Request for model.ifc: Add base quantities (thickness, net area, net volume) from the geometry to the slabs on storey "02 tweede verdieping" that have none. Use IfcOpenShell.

First a look at what the model holds.

```python
import ifcopenshell
import ifcopenshell.util.element
import ifcopenshell.util.unit

model = ifcopenshell.open("model.ifc")
print(model.schema)
for unit_type in ("LENGTHUNIT", "AREAUNIT", "VOLUMEUNIT"):
    print(unit_type, ifcopenshell.util.unit.calculate_unit_scale(model, unit_type))
storey = next(s for s in model.by_type("IfcBuildingStorey") if s.Name == "02 tweede verdieping")
slabs = [e for e in ifcopenshell.util.element.get_decomposition(storey) if e.is_a("IfcSlab")]
for e in sorted(slabs, key=lambda e: e.id()):
    print(e.id(), e.is_a(), e.Name, list(ifcopenshell.util.element.get_psets(e, qtos_only=True)), sep=" | ")
```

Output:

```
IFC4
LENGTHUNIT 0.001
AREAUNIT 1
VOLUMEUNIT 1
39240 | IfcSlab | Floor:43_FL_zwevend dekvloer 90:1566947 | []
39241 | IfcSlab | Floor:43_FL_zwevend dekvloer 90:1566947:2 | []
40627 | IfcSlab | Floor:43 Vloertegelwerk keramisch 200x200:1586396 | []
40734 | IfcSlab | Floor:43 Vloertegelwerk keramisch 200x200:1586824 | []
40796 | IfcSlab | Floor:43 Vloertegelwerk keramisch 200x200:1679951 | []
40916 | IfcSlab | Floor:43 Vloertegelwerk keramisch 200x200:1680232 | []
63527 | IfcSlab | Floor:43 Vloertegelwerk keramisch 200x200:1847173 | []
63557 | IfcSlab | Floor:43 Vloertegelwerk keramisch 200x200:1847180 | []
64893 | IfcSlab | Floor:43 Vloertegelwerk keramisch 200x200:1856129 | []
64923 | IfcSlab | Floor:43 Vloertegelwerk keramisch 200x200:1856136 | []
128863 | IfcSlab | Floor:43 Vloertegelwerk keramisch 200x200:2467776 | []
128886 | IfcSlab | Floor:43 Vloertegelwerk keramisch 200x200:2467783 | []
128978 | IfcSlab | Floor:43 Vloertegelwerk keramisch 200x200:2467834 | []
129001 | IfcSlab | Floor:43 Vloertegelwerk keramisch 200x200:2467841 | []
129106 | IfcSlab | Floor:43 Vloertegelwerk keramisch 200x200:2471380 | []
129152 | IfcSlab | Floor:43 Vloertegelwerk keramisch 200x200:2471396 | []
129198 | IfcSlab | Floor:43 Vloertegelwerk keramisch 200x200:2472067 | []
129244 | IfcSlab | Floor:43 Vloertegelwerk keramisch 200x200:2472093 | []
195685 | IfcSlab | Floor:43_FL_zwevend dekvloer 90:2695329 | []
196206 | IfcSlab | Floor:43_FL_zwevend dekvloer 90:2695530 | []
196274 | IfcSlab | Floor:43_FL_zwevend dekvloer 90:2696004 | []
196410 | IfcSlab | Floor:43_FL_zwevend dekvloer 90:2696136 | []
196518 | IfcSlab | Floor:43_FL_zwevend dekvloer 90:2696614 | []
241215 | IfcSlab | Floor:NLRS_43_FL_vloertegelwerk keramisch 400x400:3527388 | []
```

```python
import ifcopenshell
import ifcopenshell.api.pset
import ifcopenshell.geom
import ifcopenshell.util.element
import ifcopenshell.util.shape
import ifcopenshell.util.unit

model = ifcopenshell.open("model.ifc")
unit_scale = ifcopenshell.util.unit.calculate_unit_scale(model)
area_scale = ifcopenshell.util.unit.calculate_unit_scale(model, "AREAUNIT")
volume_scale = ifcopenshell.util.unit.calculate_unit_scale(model, "VOLUMEUNIT")
settings = ifcopenshell.geom.settings()

storey = next(s for s in model.by_type("IfcBuildingStorey") if s.Name == "02 tweede verdieping")
slabs = [e for e in ifcopenshell.util.element.get_decomposition(storey) if e.is_a("IfcSlab")]

for e in sorted(slabs, key=lambda e: e.id()):
    if ifcopenshell.util.element.get_psets(e, qtos_only=True, should_inherit=False):
        continue
    # Geometry comes back in metres, in the element's own axes.
    shape = ifcopenshell.geom.create_shape(settings, e)
    values = {
        "Width": ifcopenshell.util.shape.get_z(shape.geometry) / unit_scale,
        "NetArea": ifcopenshell.util.shape.get_footprint_area(shape.geometry) / area_scale,
        "NetVolume": ifcopenshell.util.shape.get_volume(shape.geometry) / volume_scale,
    }
    qto = ifcopenshell.api.pset.add_qto(model, product=e, name="Qto_SlabBaseQuantities")
    ifcopenshell.api.pset.edit_qto(model, qto=qto, properties=values)
    print(e.id(), {k: round(v, 3) for k, v in values.items()})

model.write("model_updated.ifc")
```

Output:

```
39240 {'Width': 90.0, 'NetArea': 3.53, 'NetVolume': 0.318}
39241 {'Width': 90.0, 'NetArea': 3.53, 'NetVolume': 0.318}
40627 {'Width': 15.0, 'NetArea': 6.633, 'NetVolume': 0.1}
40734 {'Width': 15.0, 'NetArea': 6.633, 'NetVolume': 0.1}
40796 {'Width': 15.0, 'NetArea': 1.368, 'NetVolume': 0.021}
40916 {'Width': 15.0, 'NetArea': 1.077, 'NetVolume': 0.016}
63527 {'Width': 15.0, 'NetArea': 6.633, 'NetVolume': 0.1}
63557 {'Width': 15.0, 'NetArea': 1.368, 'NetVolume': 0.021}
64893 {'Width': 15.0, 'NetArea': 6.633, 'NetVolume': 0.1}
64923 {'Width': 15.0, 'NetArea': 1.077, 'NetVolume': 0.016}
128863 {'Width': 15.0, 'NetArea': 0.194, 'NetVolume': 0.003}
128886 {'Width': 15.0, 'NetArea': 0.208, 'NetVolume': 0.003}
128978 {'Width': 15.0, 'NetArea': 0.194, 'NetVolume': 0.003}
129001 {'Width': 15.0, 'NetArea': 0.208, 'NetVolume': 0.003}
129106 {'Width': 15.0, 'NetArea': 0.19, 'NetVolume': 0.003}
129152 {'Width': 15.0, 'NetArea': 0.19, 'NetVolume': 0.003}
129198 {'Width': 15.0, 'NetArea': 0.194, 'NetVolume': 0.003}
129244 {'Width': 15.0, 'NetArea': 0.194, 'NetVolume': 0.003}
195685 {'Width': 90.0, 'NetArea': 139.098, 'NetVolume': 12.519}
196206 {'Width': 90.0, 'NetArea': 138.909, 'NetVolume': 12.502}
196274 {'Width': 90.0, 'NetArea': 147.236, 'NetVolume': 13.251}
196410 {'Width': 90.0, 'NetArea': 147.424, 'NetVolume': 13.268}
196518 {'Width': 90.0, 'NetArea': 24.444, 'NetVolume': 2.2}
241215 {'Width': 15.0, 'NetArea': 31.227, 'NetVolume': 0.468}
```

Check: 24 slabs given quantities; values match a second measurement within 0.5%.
